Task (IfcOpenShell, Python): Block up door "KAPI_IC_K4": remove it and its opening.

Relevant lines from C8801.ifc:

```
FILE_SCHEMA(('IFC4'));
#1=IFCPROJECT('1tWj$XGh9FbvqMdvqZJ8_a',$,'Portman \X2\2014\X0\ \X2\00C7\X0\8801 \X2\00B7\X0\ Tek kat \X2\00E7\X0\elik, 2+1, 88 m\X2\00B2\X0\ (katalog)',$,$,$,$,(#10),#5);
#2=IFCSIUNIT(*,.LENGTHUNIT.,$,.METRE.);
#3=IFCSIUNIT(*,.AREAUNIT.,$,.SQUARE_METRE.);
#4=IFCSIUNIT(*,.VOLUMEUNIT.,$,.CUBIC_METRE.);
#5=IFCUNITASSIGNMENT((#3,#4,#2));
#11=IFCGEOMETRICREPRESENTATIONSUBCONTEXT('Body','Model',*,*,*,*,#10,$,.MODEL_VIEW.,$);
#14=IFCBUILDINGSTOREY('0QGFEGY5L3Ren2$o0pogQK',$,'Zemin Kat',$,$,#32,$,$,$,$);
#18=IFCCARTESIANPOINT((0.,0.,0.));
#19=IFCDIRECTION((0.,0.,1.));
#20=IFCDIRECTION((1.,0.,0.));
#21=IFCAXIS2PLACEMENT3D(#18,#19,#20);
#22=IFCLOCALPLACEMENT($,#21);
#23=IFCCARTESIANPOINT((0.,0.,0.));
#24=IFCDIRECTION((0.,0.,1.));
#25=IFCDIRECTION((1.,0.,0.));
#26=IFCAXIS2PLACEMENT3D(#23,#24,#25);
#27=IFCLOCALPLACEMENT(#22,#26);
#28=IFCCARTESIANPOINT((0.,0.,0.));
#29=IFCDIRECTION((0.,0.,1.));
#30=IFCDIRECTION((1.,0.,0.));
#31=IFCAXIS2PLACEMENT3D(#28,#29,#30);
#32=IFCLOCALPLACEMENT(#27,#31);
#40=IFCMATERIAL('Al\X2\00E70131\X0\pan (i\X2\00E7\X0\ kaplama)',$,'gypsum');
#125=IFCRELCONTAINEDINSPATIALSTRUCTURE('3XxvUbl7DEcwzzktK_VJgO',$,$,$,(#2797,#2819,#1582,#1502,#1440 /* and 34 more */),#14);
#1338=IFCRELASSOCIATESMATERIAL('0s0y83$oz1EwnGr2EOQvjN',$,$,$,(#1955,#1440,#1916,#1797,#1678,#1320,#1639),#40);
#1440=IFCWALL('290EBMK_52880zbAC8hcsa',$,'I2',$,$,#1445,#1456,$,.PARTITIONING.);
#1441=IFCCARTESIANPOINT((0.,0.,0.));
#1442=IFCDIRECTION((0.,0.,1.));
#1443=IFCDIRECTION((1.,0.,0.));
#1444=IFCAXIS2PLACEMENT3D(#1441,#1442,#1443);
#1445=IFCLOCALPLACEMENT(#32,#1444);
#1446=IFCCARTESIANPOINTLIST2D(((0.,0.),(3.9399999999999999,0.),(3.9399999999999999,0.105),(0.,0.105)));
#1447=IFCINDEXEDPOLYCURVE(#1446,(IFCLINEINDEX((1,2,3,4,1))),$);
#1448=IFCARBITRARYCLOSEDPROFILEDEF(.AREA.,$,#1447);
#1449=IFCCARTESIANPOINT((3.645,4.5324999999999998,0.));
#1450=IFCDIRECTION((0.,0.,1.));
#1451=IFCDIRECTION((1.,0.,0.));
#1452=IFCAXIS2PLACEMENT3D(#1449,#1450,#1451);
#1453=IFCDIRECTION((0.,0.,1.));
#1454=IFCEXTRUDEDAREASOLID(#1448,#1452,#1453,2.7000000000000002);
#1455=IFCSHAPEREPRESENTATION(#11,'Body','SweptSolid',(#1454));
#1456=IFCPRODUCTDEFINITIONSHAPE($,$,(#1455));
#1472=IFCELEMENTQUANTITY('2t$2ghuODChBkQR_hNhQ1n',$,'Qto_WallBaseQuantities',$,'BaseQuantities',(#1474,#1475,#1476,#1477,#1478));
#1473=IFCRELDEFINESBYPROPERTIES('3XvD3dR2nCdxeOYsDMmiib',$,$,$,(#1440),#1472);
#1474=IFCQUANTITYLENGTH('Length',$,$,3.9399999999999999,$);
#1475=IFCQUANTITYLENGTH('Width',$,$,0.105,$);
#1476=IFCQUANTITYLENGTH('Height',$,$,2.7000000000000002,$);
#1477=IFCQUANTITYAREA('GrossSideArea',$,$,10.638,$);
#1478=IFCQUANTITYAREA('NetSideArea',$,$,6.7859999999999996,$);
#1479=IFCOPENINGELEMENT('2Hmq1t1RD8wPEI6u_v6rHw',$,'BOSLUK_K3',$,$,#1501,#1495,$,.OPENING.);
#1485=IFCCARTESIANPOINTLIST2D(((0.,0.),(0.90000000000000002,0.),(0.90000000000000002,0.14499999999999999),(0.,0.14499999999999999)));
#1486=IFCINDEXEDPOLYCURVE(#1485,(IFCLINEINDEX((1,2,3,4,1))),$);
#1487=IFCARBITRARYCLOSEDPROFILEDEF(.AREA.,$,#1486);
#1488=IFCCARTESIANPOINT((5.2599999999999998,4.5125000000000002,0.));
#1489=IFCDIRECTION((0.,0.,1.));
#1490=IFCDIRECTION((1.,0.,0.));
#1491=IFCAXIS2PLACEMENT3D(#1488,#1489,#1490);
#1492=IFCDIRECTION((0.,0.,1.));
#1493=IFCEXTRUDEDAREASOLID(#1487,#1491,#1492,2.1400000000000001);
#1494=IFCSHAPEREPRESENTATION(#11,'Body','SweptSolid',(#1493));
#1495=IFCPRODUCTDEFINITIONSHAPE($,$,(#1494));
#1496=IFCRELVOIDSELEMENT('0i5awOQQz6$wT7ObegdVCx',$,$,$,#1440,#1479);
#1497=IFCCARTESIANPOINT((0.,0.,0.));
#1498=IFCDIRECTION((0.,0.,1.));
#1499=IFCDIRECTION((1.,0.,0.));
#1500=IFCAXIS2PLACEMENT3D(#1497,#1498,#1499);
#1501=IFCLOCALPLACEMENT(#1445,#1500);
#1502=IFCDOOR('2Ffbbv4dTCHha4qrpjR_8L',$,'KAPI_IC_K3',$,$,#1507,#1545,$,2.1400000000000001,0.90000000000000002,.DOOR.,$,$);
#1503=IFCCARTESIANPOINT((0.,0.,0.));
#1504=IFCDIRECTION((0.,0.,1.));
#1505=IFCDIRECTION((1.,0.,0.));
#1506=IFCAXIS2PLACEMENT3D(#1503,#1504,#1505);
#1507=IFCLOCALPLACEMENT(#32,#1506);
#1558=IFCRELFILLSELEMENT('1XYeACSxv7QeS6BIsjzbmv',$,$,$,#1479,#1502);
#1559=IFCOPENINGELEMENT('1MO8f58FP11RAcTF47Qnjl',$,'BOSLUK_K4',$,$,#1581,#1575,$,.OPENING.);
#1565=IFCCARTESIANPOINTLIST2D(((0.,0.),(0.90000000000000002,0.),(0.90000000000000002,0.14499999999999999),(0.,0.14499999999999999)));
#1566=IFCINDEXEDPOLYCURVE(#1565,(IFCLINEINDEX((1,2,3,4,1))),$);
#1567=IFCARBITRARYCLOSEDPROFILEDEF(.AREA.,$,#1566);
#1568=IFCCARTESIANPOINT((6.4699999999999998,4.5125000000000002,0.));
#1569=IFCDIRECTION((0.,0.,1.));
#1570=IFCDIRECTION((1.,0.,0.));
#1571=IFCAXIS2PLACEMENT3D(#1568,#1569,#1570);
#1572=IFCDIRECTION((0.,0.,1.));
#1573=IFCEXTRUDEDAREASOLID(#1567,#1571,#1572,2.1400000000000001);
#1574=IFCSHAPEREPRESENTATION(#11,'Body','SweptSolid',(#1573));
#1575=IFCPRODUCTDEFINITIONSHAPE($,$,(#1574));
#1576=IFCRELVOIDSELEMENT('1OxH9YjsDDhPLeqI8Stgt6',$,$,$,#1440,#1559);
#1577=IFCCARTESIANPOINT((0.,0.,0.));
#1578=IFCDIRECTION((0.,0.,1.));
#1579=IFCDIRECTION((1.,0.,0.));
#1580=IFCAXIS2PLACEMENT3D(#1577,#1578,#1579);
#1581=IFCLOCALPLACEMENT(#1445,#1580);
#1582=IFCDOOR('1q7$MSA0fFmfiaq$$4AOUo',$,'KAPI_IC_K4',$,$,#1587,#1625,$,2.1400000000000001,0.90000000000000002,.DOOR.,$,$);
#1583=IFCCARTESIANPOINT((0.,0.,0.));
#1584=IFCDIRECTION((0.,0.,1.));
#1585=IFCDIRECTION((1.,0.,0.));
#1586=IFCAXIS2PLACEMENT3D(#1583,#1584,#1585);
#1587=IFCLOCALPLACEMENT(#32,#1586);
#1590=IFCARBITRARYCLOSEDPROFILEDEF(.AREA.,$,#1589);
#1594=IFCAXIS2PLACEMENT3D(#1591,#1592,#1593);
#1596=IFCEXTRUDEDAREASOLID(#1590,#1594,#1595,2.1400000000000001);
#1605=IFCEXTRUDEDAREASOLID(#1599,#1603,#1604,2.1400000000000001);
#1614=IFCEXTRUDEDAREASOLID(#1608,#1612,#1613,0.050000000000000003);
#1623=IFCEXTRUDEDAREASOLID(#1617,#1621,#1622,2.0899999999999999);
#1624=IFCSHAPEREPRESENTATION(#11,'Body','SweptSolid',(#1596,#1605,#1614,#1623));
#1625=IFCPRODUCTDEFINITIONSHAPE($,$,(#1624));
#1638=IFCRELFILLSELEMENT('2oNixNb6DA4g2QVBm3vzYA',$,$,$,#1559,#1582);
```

```python
import ifcopenshell
import ifcopenshell.api.feature
import ifcopenshell.api.pset
import ifcopenshell.api.root
import ifcopenshell.geom
import ifcopenshell.util.element
import ifcopenshell.util.shape
import ifcopenshell.util.unit

model = ifcopenshell.open("C8801.ifc")
area_scale = ifcopenshell.util.unit.calculate_unit_scale(model, "AREAUNIT")
settings = ifcopenshell.geom.settings()


def volume(element):
    """Net volume in cubic metres, openings subtracted."""
    shape = ifcopenshell.geom.create_shape(settings, element)
    return ifcopenshell.util.shape.get_volume(shape.geometry)


door = model.by_id(1582)
opening = door.FillsVoids[0].RelatingOpeningElement
wall = opening.VoidsElements[0].RelatingBuildingElement
before = volume(wall)

ifcopenshell.api.root.remove_product(model, product=door)
ifcopenshell.api.feature.remove_feature(model, feature=opening)

after = volume(wall)
thickness = 0.105  # wall thickness in metres

# Update the wall's stored quantities.
qto = model.by_id(ifcopenshell.util.element.get_pset(wall, "Qto_WallBaseQuantities", should_inherit=False)["id"])
ifcopenshell.api.pset.edit_qto(model, qto=qto, properties={"NetSideArea": after / thickness / area_scale})

print(f"wall volume {before:.3f} -> {after:.3f} m3")

model.write("C8801_v2.ifc")
```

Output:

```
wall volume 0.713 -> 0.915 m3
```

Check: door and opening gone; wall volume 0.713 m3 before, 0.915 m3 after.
